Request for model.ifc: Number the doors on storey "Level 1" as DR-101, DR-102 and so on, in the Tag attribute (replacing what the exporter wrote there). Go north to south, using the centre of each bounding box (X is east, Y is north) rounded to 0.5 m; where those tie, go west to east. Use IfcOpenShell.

First a look at what the model holds.

```python
import ifcopenshell
import ifcopenshell.util.element
import ifcopenshell.util.placement

model = ifcopenshell.open("model.ifc")
print(model.schema)
storey = next(s for s in model.by_type("IfcBuildingStorey") if s.Name == "Level 1")
doors = [e for e in ifcopenshell.util.element.get_decomposition(storey) if e.is_a("IfcDoor")]
for e in sorted(doors, key=lambda e: e.id()):
    origin = ifcopenshell.util.placement.get_local_placement(e.ObjectPlacement)[:3, 3]
    print(e.id(), e.Tag, e.Name, origin.round(2) + 0.0, sep=" | ")
```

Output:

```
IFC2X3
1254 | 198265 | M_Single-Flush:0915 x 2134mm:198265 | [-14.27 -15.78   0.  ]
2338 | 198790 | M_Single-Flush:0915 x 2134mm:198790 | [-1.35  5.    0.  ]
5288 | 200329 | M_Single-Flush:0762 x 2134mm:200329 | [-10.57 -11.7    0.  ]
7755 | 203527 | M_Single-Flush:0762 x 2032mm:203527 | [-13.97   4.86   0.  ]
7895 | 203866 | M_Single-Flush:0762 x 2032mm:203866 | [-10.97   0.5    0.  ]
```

```python
import ifcopenshell
import ifcopenshell.geom
import ifcopenshell.util.element
import ifcopenshell.util.shape

model = ifcopenshell.open("model.ifc")
settings = ifcopenshell.geom.settings()
settings.set("use-world-coords", True)


def centre(element):
    shape = ifcopenshell.geom.create_shape(settings, element)
    return ifcopenshell.util.shape.get_bbox_centroid(shape.geometry)


storey = next(s for s in model.by_type("IfcBuildingStorey") if s.Name == "Level 1")
doors = [e for e in ifcopenshell.util.element.get_decomposition(storey) if e.is_a("IfcDoor")]

# Insertion points can sit at a corner or the storey origin, so sort by the geometry (in metres).
centres = {e: centre(e) for e in doors}
doors.sort(key=lambda e: (-round(centres[e][1] / 0.5), centres[e][0]))

for i, e in enumerate(doors, start=1):
    number = f"DR-1{i:02d}"
    e.Tag = number
    print(e.id(), number)

model.write("model_rev.ifc")
```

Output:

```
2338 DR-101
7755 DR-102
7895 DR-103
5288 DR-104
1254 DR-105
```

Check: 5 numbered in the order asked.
